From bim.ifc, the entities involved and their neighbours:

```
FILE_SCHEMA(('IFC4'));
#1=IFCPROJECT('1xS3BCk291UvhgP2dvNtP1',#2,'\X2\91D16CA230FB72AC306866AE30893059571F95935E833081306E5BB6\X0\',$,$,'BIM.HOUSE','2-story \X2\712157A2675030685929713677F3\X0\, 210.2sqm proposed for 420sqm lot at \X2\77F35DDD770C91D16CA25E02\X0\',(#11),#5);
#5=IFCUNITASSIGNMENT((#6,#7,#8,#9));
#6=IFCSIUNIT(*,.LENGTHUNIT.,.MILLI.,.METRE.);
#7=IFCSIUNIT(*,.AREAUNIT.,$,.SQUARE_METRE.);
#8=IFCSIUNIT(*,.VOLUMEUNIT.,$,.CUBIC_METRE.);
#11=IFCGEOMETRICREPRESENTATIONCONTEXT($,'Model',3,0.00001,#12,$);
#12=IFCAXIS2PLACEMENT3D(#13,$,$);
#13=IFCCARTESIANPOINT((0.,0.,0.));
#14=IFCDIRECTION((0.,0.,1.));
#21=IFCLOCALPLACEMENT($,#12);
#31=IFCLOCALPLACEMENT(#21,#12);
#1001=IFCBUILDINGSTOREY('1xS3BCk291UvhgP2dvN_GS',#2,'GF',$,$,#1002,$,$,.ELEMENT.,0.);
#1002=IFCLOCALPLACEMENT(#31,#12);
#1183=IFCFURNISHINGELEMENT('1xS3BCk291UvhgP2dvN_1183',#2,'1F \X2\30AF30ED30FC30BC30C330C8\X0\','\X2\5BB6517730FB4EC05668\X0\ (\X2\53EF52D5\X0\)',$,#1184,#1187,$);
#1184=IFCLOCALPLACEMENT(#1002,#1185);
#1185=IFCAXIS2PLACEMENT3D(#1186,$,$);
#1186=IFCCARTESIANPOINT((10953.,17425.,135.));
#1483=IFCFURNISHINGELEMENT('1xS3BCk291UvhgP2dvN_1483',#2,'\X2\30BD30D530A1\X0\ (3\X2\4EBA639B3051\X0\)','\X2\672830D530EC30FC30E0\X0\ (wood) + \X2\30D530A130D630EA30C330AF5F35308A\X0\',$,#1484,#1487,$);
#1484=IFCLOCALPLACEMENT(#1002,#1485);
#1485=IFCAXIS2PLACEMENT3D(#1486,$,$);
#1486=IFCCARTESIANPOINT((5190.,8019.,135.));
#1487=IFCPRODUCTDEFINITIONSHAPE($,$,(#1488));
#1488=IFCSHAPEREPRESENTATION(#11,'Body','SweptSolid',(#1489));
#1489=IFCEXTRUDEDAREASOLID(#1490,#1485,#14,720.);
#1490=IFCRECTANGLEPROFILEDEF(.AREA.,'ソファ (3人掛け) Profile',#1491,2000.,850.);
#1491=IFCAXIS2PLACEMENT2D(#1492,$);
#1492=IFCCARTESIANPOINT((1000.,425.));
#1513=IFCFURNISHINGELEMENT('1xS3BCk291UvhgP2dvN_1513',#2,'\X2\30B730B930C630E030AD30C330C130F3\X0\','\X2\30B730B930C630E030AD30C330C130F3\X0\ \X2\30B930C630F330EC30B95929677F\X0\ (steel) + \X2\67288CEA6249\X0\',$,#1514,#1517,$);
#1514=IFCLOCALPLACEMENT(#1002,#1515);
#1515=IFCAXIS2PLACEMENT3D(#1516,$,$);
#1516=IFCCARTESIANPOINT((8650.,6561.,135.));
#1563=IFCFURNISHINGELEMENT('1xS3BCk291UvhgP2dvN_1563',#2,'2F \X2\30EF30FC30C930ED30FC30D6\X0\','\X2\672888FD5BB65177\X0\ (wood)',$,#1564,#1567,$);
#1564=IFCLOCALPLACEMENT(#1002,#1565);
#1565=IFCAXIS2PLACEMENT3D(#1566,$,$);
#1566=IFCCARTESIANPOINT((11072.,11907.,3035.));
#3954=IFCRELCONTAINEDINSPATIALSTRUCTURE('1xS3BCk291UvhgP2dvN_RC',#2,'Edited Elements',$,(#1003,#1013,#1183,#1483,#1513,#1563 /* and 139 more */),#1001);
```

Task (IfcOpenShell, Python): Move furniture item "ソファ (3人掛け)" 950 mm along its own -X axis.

```python
import ifcopenshell
import ifcopenshell.api.geometry
import ifcopenshell.util.placement

model = ifcopenshell.open("bim.ifc")

item = model.by_guid("1xS3BCk291UvhgP2dvN_1483")
matrix = ifcopenshell.util.placement.get_local_placement(item.ObjectPlacement)
matrix[:3, 3] -= matrix[:3, 0] * 950.0
ifcopenshell.api.geometry.edit_object_placement(model, product=item, matrix=matrix, is_si=False)

print(ifcopenshell.util.placement.get_local_placement(item.ObjectPlacement).round(3) + 0.0)

model.write("bim-out.ifc")
```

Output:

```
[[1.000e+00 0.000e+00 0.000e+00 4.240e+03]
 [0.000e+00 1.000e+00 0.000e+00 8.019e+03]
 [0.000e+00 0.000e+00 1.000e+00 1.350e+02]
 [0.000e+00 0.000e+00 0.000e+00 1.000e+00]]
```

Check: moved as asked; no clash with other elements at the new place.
